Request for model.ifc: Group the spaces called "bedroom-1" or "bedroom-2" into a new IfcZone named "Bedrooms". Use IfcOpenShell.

First a look at what the model holds.

```python
import ifcopenshell

model = ifcopenshell.open("model.ifc")
print(model.schema)
seen = {}
for space in model.by_type("IfcSpace"):
    seen[space.Name] = seen.get(space.Name, 0) + 1
for name, count in sorted(seen.items(), key=str):
    print(count, "x", name)
print("zones:", [z.Name for z in model.by_type("IfcZone")][:20])
```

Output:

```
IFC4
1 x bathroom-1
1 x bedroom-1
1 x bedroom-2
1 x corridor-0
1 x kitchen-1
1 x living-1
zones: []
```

```python
import ifcopenshell
import ifcopenshell.api.group
import ifcopenshell.api.root

model = ifcopenshell.open("model.ifc")

names = {"bedroom-1", "bedroom-2"}
spaces = [s for s in model.by_type("IfcSpace") if s.Name in names]

zone = ifcopenshell.api.root.create_entity(model, ifc_class="IfcZone", name="Bedrooms")
ifcopenshell.api.group.assign_group(model, products=spaces, group=zone)
print(len(spaces), "spaces in", zone.Name)

model.write("model-out.ifc")
```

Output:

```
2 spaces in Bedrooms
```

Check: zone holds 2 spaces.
